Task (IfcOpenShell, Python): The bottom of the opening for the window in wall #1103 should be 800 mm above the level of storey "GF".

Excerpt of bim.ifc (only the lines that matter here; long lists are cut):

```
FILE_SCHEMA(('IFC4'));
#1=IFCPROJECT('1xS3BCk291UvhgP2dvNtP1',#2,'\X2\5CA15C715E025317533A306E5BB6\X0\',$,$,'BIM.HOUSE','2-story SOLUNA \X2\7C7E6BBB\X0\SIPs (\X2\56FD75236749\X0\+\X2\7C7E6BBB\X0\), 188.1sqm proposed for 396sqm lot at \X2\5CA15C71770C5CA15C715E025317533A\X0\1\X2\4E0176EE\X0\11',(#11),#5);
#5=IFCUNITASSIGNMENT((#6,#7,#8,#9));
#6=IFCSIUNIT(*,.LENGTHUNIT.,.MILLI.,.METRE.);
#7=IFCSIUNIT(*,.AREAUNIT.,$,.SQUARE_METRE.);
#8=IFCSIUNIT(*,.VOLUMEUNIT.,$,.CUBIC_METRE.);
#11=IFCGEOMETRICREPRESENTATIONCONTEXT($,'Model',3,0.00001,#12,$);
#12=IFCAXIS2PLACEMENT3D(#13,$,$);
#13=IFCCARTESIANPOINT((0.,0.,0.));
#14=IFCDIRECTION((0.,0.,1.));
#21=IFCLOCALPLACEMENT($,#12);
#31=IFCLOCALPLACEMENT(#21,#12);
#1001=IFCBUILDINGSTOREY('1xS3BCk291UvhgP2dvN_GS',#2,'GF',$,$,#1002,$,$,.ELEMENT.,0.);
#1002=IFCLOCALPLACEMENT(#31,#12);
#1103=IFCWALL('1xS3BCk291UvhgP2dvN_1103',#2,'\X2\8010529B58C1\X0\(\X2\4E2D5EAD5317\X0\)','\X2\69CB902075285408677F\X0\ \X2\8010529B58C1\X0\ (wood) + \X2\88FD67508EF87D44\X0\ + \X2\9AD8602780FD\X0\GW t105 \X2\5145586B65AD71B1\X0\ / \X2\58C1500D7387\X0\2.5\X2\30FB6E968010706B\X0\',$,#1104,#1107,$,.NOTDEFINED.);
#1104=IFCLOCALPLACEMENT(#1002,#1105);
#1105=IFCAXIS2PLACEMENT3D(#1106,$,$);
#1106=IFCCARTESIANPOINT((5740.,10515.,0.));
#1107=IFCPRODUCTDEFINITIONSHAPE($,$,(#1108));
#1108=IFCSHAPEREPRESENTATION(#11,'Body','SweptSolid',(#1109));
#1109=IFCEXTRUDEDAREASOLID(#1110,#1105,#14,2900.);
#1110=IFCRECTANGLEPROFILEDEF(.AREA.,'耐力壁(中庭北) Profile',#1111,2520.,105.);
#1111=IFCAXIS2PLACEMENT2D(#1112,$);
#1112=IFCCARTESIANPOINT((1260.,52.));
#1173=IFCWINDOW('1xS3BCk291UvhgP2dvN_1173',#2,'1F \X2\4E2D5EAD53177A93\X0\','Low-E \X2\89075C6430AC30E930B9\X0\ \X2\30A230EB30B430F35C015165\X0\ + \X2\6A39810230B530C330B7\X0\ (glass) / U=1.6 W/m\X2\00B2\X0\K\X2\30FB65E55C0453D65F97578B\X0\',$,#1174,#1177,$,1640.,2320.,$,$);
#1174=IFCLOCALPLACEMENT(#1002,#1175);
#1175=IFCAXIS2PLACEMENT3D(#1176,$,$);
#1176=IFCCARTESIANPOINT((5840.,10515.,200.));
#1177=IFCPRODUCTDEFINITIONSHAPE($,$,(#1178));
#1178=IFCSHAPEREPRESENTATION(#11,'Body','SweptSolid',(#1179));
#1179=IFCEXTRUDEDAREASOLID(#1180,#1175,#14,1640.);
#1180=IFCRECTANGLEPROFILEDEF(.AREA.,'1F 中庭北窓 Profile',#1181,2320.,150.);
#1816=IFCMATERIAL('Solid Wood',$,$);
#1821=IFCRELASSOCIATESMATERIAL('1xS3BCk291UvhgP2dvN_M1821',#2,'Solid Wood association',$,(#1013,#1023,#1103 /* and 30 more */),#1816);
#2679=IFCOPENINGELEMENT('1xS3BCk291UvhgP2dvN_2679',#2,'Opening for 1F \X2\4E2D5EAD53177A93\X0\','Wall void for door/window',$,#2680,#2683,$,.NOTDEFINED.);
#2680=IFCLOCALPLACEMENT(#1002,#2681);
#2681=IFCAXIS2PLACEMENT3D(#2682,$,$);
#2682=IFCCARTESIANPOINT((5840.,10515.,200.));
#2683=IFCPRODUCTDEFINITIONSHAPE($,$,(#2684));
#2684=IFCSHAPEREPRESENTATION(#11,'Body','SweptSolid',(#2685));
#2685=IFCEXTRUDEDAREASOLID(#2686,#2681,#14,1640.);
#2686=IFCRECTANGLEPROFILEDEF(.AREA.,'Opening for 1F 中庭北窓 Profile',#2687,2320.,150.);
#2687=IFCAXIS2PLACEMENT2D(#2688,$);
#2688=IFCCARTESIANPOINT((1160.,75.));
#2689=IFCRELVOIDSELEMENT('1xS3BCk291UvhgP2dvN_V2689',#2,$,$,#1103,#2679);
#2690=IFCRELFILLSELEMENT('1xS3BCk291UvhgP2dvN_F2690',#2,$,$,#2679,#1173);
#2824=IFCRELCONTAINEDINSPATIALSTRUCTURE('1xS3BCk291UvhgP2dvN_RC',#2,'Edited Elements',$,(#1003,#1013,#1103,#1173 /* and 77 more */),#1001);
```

```python
import numpy as np
import ifcopenshell
import ifcopenshell.api.geometry
import ifcopenshell.geom
import ifcopenshell.util.element
import ifcopenshell.util.placement
import ifcopenshell.util.shape
import ifcopenshell.util.unit

model = ifcopenshell.open("bim.ifc")
unit_scale = ifcopenshell.util.unit.calculate_unit_scale(model)

window = model.by_guid("1xS3BCk291UvhgP2dvN_1173")
opening = window.FillsVoids[0].RelatingOpeningElement
storey = ifcopenshell.util.element.get_container(window, ifc_class="IfcBuildingStorey")
level = ifcopenshell.util.placement.get_local_placement(storey.ObjectPlacement)[2, 3]

# The opening's origin need not be at the sill, so measure its lowest point.
shape = ifcopenshell.geom.create_shape(ifcopenshell.geom.settings(), opening)
bottom = ifcopenshell.util.shape.get_shape_bottom_elevation(shape, shape.geometry) / unit_scale
dz = level + 0.8 / unit_scale - bottom

shift = np.array([0.0, 0.0, dz])
# The window is not placed relative to its opening, so move both.
for product in (opening, window):
    matrix = ifcopenshell.util.placement.get_local_placement(product.ObjectPlacement)
    matrix[:3, 3] += shift
    ifcopenshell.api.geometry.edit_object_placement(model, product=product, matrix=matrix, is_si=False)

print(f"moved by {dz * unit_scale:+.3f} m")

model.write("bim_updated.ifc")
```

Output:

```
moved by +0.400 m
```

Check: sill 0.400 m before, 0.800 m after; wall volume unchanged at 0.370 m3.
